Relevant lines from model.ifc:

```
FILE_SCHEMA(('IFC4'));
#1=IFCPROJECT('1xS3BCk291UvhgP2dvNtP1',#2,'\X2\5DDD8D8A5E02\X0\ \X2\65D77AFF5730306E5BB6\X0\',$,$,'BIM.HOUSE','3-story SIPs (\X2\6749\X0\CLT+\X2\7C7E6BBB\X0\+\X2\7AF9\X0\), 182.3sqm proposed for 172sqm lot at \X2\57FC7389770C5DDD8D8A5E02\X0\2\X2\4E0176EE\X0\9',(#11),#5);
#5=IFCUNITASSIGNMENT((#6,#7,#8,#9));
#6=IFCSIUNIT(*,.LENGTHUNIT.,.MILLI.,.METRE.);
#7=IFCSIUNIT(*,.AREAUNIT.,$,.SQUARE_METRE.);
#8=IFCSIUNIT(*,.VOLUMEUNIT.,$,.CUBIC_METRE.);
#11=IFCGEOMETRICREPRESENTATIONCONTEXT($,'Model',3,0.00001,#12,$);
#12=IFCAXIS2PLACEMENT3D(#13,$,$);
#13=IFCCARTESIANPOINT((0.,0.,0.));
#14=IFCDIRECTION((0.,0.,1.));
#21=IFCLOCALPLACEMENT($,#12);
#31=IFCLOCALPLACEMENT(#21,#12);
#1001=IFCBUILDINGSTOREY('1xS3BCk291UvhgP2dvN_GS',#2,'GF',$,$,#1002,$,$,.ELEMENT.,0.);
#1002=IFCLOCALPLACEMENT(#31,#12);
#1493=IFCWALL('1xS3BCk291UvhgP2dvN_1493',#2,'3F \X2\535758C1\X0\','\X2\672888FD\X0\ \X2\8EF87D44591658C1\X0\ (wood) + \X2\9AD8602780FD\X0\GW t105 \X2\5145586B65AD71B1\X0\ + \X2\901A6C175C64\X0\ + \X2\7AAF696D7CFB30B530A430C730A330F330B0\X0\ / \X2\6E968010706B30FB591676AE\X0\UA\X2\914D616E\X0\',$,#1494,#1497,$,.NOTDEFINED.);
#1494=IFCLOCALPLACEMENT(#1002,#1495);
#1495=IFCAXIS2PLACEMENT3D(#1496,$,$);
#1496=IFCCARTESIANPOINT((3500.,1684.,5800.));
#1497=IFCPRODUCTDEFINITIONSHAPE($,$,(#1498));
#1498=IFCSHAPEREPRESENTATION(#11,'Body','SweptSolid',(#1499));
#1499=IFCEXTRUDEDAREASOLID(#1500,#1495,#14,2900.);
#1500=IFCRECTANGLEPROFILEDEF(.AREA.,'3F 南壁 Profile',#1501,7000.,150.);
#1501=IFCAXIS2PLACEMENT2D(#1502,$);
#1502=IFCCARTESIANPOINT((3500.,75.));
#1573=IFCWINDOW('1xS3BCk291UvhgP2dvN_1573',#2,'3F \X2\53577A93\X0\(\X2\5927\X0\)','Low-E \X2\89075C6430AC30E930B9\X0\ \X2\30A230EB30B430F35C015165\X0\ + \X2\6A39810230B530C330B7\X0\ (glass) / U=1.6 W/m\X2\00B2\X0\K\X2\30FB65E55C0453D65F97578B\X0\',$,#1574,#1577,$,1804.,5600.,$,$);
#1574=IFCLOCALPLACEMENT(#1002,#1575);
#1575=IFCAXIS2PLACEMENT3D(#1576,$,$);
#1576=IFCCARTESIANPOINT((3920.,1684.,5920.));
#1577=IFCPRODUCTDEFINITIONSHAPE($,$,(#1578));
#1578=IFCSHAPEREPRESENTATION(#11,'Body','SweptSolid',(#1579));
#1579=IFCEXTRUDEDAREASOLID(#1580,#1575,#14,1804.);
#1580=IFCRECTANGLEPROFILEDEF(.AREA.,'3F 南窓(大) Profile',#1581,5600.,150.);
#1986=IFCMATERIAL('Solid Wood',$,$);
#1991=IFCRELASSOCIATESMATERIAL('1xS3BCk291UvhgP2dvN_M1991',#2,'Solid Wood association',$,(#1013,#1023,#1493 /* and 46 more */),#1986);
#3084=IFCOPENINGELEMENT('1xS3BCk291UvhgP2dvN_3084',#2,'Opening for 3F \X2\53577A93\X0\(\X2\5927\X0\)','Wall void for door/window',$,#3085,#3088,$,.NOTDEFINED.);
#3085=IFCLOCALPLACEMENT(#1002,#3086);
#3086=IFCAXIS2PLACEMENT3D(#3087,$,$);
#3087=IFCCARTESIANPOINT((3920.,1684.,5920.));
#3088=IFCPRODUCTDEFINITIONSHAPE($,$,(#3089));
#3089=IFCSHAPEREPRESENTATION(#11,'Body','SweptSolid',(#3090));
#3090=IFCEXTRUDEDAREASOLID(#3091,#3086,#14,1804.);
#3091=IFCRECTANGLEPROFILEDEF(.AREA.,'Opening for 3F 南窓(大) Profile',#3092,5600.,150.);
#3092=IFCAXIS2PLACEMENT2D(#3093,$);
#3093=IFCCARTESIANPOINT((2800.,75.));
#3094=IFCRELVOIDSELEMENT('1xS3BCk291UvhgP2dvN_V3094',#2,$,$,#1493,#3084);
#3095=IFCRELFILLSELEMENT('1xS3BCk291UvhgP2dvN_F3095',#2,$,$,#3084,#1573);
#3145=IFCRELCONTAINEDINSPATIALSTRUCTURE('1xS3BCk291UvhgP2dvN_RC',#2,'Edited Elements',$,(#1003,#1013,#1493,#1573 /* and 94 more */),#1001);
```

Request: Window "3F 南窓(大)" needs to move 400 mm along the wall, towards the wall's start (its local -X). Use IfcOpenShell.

```python
import ifcopenshell
import ifcopenshell.api.geometry
import ifcopenshell.util.placement
import ifcopenshell.util.unit

model = ifcopenshell.open("model.ifc")
unit_scale = ifcopenshell.util.unit.calculate_unit_scale(model)

window = model.by_id(1573)
opening = window.FillsVoids[0].RelatingOpeningElement
wall = opening.VoidsElements[0].RelatingBuildingElement

wall_matrix = ifcopenshell.util.placement.get_local_placement(wall.ObjectPlacement)
shift = wall_matrix[:3, 0] * -0.4 / unit_scale
before = ifcopenshell.util.placement.get_local_placement(window.ObjectPlacement)[:3, 3].copy()

# The window is not placed relative to its opening, so move both.
for product in (opening, window):
    matrix = ifcopenshell.util.placement.get_local_placement(product.ObjectPlacement)
    matrix[:3, 3] += shift
    ifcopenshell.api.geometry.edit_object_placement(model, product=product, matrix=matrix, is_si=False)

after = ifcopenshell.util.placement.get_local_placement(window.ObjectPlacement)[:3, 3]
print("window moved by", (after - before).round(3) + 0.0)

model.write("model_edited.ifc")
```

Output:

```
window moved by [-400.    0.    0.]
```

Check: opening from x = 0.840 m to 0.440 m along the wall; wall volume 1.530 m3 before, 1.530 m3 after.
